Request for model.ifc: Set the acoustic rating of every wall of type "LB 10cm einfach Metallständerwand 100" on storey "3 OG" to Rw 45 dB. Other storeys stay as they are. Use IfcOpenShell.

First a look at what the model holds.

```python
import ifcopenshell
import ifcopenshell.util.element

model = ifcopenshell.open("model.ifc")
print(model.schema)
storey = next(s for s in model.by_type("IfcBuildingStorey") if s.Name == "3 OG")
walls = [e for e in ifcopenshell.util.element.get_decomposition(storey) if e.is_a("IfcWall")]
seen = {}
for e in walls:
    element_type = ifcopenshell.util.element.get_type(e)
    key = (element_type.Name if element_type != e and element_type else None, ifcopenshell.util.element.get_pset(e, "Pset_WallCommon", "AcousticRating"))
    seen[key] = seen.get(key, 0) + 1
for (name, value), count in sorted(seen.items(), key=str):
    print(count, "x", name, "|", value)
```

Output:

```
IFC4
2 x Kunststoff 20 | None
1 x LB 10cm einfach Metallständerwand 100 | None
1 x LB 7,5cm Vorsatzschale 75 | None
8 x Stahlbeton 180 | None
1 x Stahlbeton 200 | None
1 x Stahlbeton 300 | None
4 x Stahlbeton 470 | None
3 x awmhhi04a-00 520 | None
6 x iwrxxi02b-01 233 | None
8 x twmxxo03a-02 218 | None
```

```python
import ifcopenshell
import ifcopenshell.api.pset
import ifcopenshell.util.element

model = ifcopenshell.open("model.ifc")

storey = next(s for s in model.by_type("IfcBuildingStorey") if s.Name == "3 OG")
walls = [e for e in ifcopenshell.util.element.get_decomposition(storey) if e.is_a("IfcWall")]

count = 0
for e in walls:
    element_type = ifcopenshell.util.element.get_type(e)
    if element_type in (None, e) or element_type.Name != "LB 10cm einfach Metallständerwand 100":
        continue
    # add_pset returns the element's existing set when there is one.
    pset = ifcopenshell.api.pset.add_pset(model, product=e, name="Pset_WallCommon")
    ifcopenshell.api.pset.edit_pset(model, pset=pset, properties={"AcousticRating": "Rw 45 dB"})
    count += 1

print(count, "walls updated")

model.write("model_updated.ifc")
```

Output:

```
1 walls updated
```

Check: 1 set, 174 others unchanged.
